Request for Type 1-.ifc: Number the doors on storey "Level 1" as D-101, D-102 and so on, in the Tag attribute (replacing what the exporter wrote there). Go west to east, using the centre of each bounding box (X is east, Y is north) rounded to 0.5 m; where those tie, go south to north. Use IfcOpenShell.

First a look at what the model holds.

```python
import ifcopenshell
import ifcopenshell.util.element
import ifcopenshell.util.placement

model = ifcopenshell.open("Type 1-.ifc")
print(model.schema)
storey = next(s for s in model.by_type("IfcBuildingStorey") if s.Name == "Level 1")
doors = [e for e in ifcopenshell.util.element.get_decomposition(storey) if e.is_a("IfcDoor")]
for e in sorted(doors, key=lambda e: e.id()):
    origin = ifcopenshell.util.placement.get_local_placement(e.ObjectPlacement)[:3, 3]
    print(e.id(), e.Tag, e.Name, origin.round(2) + 0.0, sep=" | ")
```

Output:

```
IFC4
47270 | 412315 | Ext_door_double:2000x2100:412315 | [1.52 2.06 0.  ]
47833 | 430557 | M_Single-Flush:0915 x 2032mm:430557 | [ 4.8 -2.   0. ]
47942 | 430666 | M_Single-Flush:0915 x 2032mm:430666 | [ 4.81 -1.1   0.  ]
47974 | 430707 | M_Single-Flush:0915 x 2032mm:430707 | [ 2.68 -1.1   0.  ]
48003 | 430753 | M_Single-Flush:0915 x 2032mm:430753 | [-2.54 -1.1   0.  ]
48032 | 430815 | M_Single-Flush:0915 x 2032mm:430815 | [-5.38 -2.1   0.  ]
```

```python
import ifcopenshell
import ifcopenshell.geom
import ifcopenshell.util.element
import ifcopenshell.util.shape

model = ifcopenshell.open("Type 1-.ifc")
settings = ifcopenshell.geom.settings()
settings.set("use-world-coords", True)


def centre(element):
    shape = ifcopenshell.geom.create_shape(settings, element)
    return ifcopenshell.util.shape.get_bbox_centroid(shape.geometry)


storey = next(s for s in model.by_type("IfcBuildingStorey") if s.Name == "Level 1")
doors = [e for e in ifcopenshell.util.element.get_decomposition(storey) if e.is_a("IfcDoor")]

# Insertion points can sit at a corner or the storey origin, so sort by the geometry (in metres).
centres = {e: centre(e) for e in doors}
doors.sort(key=lambda e: (round(centres[e][0] / 0.5), centres[e][1]))

for i, e in enumerate(doors, start=1):
    number = f"D-1{i:02d}"
    e.Tag = number
    print(e.id(), number)

model.write("Type 1-_rev.ifc")
```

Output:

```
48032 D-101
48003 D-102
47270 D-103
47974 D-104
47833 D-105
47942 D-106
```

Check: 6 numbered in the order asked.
